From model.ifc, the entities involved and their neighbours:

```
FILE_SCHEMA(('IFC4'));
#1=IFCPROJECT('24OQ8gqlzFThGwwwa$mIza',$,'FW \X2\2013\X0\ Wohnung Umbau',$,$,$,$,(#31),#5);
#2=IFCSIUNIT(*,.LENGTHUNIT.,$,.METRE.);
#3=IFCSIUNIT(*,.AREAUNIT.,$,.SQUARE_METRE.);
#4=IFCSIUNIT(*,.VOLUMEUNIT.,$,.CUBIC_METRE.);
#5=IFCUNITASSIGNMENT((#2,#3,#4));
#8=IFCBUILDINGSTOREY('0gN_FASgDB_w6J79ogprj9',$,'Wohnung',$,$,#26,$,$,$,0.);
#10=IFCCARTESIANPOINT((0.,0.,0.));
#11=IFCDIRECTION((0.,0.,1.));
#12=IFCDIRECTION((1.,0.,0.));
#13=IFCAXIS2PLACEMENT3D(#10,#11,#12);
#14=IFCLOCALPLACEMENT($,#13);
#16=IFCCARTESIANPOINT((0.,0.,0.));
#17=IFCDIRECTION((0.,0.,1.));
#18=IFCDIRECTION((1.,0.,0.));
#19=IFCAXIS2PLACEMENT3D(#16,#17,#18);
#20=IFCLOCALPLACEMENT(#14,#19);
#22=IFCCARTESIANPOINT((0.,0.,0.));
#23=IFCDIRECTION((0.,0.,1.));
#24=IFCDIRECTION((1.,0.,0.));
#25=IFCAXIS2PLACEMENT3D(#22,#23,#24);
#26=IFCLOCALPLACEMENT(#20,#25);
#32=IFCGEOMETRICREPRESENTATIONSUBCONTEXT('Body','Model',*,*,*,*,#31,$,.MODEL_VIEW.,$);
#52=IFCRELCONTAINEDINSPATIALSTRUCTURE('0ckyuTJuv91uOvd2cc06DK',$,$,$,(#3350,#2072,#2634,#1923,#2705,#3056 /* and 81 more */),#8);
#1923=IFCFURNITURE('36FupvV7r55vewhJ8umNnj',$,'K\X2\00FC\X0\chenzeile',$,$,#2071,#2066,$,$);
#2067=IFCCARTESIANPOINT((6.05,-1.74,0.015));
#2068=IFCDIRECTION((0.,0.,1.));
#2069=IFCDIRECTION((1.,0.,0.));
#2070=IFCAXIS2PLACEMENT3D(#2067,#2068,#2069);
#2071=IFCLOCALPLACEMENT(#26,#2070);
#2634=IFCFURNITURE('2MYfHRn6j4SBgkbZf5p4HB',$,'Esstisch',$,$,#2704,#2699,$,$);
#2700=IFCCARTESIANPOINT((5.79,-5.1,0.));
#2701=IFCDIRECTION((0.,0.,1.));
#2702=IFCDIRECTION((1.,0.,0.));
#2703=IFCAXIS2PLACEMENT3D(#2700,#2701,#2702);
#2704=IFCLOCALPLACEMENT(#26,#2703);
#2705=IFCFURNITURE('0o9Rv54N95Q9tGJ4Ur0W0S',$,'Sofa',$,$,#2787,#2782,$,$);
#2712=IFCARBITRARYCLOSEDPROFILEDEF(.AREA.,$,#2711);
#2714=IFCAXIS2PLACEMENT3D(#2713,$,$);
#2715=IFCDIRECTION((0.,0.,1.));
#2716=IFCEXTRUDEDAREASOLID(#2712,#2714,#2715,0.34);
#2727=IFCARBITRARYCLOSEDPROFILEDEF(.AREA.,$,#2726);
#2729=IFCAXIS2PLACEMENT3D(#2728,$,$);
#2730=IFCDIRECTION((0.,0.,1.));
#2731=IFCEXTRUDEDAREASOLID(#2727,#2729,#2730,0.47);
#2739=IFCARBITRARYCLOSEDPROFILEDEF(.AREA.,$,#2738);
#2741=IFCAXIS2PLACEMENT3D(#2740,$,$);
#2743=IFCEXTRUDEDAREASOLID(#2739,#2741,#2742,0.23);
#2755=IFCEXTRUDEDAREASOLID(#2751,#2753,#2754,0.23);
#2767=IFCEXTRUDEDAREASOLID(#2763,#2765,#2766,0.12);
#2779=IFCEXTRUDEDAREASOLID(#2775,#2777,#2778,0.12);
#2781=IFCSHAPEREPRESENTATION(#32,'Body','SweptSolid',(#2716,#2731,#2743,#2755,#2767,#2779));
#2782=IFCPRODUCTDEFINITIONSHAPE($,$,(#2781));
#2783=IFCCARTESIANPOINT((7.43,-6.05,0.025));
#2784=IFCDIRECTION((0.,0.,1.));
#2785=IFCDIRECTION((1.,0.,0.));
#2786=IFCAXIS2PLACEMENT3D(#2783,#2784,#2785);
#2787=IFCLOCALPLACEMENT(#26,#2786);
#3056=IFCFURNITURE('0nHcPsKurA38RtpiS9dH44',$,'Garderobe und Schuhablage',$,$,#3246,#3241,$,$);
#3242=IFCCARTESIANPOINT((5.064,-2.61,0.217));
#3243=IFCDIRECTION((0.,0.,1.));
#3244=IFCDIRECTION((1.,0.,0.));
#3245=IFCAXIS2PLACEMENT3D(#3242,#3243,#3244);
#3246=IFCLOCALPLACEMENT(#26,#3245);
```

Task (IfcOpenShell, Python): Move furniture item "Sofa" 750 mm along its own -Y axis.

```python
import ifcopenshell
import ifcopenshell.api.geometry
import ifcopenshell.util.placement
import ifcopenshell.util.unit

model = ifcopenshell.open("model.ifc")
unit_scale = ifcopenshell.util.unit.calculate_unit_scale(model)

item = model.by_guid("0o9Rv54N95Q9tGJ4Ur0W0S")
matrix = ifcopenshell.util.placement.get_local_placement(item.ObjectPlacement)
matrix[:3, 3] -= matrix[:3, 1] * 0.75 / unit_scale
ifcopenshell.api.geometry.edit_object_placement(model, product=item, matrix=matrix, is_si=False)

print(ifcopenshell.util.placement.get_local_placement(item.ObjectPlacement).round(3) + 0.0)

model.write("model_rev.ifc")
```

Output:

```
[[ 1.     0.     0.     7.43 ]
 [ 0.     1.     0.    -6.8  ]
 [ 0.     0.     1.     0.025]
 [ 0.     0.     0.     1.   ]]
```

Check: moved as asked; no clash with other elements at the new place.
